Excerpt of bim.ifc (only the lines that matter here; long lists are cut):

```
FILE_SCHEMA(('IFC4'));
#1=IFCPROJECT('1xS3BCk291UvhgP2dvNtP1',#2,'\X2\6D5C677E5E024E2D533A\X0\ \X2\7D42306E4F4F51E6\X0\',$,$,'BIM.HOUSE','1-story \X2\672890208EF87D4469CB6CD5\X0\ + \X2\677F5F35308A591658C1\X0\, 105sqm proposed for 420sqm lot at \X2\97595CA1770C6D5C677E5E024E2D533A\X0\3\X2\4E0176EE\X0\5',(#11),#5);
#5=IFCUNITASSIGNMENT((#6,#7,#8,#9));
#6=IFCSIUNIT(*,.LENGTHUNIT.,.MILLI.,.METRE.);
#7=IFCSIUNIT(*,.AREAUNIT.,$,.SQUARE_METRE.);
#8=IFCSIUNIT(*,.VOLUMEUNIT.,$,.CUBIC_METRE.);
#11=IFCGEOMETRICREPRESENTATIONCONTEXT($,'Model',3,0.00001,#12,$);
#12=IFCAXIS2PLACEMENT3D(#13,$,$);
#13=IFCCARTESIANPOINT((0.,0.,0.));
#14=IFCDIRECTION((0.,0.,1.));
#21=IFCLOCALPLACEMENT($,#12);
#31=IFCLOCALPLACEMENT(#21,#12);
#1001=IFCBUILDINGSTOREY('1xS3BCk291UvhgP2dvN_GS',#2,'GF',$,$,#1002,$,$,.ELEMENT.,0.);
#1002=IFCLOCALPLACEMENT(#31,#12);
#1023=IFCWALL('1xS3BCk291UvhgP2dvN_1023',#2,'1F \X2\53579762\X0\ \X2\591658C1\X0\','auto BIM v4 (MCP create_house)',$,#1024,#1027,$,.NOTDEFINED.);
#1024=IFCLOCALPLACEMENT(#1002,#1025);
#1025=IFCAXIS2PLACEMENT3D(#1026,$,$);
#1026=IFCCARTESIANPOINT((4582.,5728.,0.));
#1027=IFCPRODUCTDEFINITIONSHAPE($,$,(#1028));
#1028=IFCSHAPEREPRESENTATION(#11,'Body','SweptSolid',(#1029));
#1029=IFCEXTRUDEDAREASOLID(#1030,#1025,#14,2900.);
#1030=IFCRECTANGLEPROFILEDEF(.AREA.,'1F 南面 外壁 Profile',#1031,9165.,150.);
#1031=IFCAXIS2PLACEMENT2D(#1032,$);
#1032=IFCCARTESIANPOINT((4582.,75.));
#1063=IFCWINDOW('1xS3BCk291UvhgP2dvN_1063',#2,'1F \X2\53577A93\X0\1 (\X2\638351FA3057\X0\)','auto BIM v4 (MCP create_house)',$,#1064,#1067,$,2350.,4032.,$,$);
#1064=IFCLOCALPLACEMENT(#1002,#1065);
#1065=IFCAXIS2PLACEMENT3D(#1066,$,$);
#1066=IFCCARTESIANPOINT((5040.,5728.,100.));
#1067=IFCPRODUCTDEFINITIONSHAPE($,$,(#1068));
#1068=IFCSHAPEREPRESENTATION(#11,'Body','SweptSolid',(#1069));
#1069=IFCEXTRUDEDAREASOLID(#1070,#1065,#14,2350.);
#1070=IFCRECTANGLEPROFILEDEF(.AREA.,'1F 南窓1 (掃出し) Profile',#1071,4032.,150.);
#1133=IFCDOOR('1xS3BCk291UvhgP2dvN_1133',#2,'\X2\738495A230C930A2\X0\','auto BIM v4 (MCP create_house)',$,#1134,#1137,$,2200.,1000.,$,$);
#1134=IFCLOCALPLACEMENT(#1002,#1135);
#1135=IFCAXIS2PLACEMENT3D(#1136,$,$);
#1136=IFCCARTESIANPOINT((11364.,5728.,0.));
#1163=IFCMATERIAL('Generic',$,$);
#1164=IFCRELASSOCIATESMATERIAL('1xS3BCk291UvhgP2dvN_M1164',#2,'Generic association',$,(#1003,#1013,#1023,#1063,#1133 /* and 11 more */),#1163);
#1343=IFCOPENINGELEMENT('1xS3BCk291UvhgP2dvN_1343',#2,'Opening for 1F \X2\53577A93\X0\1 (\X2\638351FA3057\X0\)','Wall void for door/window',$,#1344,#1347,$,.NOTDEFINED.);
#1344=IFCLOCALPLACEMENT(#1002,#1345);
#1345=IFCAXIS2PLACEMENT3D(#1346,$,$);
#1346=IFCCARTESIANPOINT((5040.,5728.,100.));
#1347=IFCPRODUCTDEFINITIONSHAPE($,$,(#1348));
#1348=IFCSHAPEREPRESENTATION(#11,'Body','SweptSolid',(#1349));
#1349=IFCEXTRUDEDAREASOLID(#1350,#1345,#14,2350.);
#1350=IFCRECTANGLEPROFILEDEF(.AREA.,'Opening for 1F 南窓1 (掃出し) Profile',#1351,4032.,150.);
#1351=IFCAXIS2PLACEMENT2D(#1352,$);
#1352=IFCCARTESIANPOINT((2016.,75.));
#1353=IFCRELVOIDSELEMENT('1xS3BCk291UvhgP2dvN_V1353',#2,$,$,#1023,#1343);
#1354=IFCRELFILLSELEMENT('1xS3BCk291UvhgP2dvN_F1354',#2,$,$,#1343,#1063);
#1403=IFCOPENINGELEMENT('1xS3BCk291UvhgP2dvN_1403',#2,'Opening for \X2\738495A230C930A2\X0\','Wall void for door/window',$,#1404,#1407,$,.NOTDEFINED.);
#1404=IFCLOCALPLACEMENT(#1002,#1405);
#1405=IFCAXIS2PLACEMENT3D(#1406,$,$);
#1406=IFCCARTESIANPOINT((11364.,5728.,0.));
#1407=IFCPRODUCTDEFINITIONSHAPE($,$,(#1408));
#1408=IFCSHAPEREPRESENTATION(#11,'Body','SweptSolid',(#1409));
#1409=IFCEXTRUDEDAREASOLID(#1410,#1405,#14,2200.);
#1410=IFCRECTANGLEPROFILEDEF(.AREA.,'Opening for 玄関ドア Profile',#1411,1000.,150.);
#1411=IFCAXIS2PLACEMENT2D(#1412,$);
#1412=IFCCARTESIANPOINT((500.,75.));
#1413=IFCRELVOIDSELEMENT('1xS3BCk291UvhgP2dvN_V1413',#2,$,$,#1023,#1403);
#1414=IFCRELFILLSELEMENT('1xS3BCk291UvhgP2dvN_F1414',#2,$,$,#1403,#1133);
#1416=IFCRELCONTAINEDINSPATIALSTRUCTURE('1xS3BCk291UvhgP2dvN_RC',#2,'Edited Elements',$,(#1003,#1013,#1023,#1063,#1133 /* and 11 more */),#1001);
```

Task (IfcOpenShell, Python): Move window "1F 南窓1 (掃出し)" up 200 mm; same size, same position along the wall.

```python
import numpy as np
import ifcopenshell
import ifcopenshell.api.geometry
import ifcopenshell.util.placement
import ifcopenshell.util.unit

model = ifcopenshell.open("bim.ifc")
unit_scale = ifcopenshell.util.unit.calculate_unit_scale(model)

window = model.by_id(1063)
opening = window.FillsVoids[0].RelatingOpeningElement
dz = 0.2 / unit_scale

shift = np.array([0.0, 0.0, dz])
# The window is not placed relative to its opening, so move both.
for product in (opening, window):
    matrix = ifcopenshell.util.placement.get_local_placement(product.ObjectPlacement)
    matrix[:3, 3] += shift
    ifcopenshell.api.geometry.edit_object_placement(model, product=product, matrix=matrix, is_si=False)

print(f"moved by {dz * unit_scale:+.3f} m")

model.write("bim_updated.ifc")
```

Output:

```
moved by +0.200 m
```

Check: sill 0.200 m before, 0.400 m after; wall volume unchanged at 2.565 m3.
